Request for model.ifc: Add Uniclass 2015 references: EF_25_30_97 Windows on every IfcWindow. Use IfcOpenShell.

First a look at what the model holds.

```python
import ifcopenshell

model = ifcopenshell.open("model.ifc")
print(model.schema)
print("classifications:", [c.Name for c in model.by_type("IfcClassification")])
for ifc_class in ("IfcDoor", "IfcRoof", "IfcStair", "IfcWall", "IfcWindow"):
    print(ifc_class, len(model.by_type(ifc_class)))
```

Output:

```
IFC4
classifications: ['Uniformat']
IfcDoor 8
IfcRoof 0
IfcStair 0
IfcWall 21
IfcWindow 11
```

```python
import ifcopenshell
import ifcopenshell.api.classification

model = ifcopenshell.open("model.ifc")

system = ifcopenshell.api.classification.add_classification(model, classification="Uniclass 2015")

codes = {
    "IfcWindow": ("EF_25_30_97", "Windows"),
}
for ifc_class, (code, name) in codes.items():
    products = model.by_type(ifc_class)
    ifcopenshell.api.classification.add_reference(
        model, products=products, classification=system, identification=code, name=name
    )
    print(code, len(products))

model.write("model_updated.ifc")
```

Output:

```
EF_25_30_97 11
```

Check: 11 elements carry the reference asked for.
